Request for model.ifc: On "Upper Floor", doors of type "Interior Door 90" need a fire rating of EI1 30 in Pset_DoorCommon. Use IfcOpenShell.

First a look at what the model holds.

```python
import ifcopenshell
import ifcopenshell.util.element

model = ifcopenshell.open("model.ifc")
print(model.schema)
storey = next(s for s in model.by_type("IfcBuildingStorey") if s.Name == "Upper Floor")
doors = [e for e in ifcopenshell.util.element.get_decomposition(storey) if e.is_a("IfcDoor")]
seen = {}
for e in doors:
    element_type = ifcopenshell.util.element.get_type(e)
    key = (element_type.Name if element_type != e and element_type else None, ifcopenshell.util.element.get_pset(e, "Pset_DoorCommon", "FireRating"))
    seen[key] = seen.get(key, 0) + 1
for (name, value), count in sorted(seen.items(), key=str):
    print(count, "x", name, "|", value)
```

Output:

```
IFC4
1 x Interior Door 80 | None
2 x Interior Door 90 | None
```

```python
import ifcopenshell
import ifcopenshell.api.pset
import ifcopenshell.util.element

model = ifcopenshell.open("model.ifc")

storey = next(s for s in model.by_type("IfcBuildingStorey") if s.Name == "Upper Floor")
doors = [e for e in ifcopenshell.util.element.get_decomposition(storey) if e.is_a("IfcDoor")]

count = 0
for e in doors:
    element_type = ifcopenshell.util.element.get_type(e)
    if element_type in (None, e) or element_type.Name != "Interior Door 90":
        continue
    # add_pset returns the element's existing set when there is one.
    pset = ifcopenshell.api.pset.add_pset(model, product=e, name="Pset_DoorCommon")
    ifcopenshell.api.pset.edit_pset(model, pset=pset, properties={"FireRating": "EI1 30"})
    count += 1

print(count, "doors updated")

model.write("model_rev.ifc")
```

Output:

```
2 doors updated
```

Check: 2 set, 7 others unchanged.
